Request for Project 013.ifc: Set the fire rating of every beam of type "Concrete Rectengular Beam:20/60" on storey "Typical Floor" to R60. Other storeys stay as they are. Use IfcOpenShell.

First a look at what the model holds.

```python
import ifcopenshell
import ifcopenshell.util.element

model = ifcopenshell.open("Project 013.ifc")
print(model.schema)
storey = next(s for s in model.by_type("IfcBuildingStorey") if s.Name == "Typical Floor")
beams = [e for e in ifcopenshell.util.element.get_decomposition(storey) if e.is_a("IfcBeam")]
seen = {}
for e in beams:
    element_type = ifcopenshell.util.element.get_type(e)
    key = (element_type.Name if element_type != e and element_type else None, ifcopenshell.util.element.get_pset(e, "Pset_BeamCommon", "FireRating"))
    seen[key] = seen.get(key, 0) + 1
for (name, value), count in sorted(seen.items(), key=str):
    print(count, "x", name, "|", value)
```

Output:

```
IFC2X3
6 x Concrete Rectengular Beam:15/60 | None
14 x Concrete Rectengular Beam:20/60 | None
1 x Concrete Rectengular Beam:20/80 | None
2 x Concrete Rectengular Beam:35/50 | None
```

```python
import ifcopenshell
import ifcopenshell.api.pset
import ifcopenshell.util.element

model = ifcopenshell.open("Project 013.ifc")

storey = next(s for s in model.by_type("IfcBuildingStorey") if s.Name == "Typical Floor")
beams = [e for e in ifcopenshell.util.element.get_decomposition(storey) if e.is_a("IfcBeam")]

count = 0
for e in beams:
    element_type = ifcopenshell.util.element.get_type(e)
    if element_type in (None, e) or element_type.Name != "Concrete Rectengular Beam:20/60":
        continue
    # add_pset returns the element's existing set when there is one.
    pset = ifcopenshell.api.pset.add_pset(model, product=e, name="Pset_BeamCommon")
    ifcopenshell.api.pset.edit_pset(model, pset=pset, properties={"FireRating": "R60"})
    count += 1

print(count, "beams updated")

model.write("Project 013_updated.ifc")
```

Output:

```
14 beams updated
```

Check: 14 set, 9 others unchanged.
